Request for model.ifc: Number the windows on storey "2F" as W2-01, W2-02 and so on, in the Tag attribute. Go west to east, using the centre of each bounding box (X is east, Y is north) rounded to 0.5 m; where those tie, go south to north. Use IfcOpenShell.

First a look at what the model holds.

```python
import ifcopenshell
import ifcopenshell.util.element
import ifcopenshell.util.placement

model = ifcopenshell.open("model.ifc")
print(model.schema)
storey = next(s for s in model.by_type("IfcBuildingStorey") if s.Name == "2F")
windows = [e for e in ifcopenshell.util.element.get_decomposition(storey) if e.is_a("IfcWindow")]
for e in sorted(windows, key=lambda e: e.id()):
    origin = ifcopenshell.util.placement.get_local_placement(e.ObjectPlacement)[:3, 3]
    print(e.id(), e.Tag, e.Name, origin.round(2) + 0.0, sep=" | ")
```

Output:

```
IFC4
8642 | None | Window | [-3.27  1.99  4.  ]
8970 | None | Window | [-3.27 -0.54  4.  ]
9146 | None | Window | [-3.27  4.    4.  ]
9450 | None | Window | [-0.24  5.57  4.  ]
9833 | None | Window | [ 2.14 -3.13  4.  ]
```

```python
import ifcopenshell
import ifcopenshell.geom
import ifcopenshell.util.element
import ifcopenshell.util.shape

model = ifcopenshell.open("model.ifc")
settings = ifcopenshell.geom.settings()
settings.set("use-world-coords", True)


def centre(element):
    shape = ifcopenshell.geom.create_shape(settings, element)
    return ifcopenshell.util.shape.get_bbox_centroid(shape.geometry)


storey = next(s for s in model.by_type("IfcBuildingStorey") if s.Name == "2F")
windows = [e for e in ifcopenshell.util.element.get_decomposition(storey) if e.is_a("IfcWindow")]

# Insertion points can sit at a corner or the storey origin, so sort by the geometry (in metres).
centres = {e: centre(e) for e in windows}
windows.sort(key=lambda e: (round(centres[e][0] / 0.5), centres[e][1]))

for i, e in enumerate(windows, start=1):
    number = f"W2-{i:02d}"
    e.Tag = number
    print(e.id(), number)

model.write("model_updated.ifc")
```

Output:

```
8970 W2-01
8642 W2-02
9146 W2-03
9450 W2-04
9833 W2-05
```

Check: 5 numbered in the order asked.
